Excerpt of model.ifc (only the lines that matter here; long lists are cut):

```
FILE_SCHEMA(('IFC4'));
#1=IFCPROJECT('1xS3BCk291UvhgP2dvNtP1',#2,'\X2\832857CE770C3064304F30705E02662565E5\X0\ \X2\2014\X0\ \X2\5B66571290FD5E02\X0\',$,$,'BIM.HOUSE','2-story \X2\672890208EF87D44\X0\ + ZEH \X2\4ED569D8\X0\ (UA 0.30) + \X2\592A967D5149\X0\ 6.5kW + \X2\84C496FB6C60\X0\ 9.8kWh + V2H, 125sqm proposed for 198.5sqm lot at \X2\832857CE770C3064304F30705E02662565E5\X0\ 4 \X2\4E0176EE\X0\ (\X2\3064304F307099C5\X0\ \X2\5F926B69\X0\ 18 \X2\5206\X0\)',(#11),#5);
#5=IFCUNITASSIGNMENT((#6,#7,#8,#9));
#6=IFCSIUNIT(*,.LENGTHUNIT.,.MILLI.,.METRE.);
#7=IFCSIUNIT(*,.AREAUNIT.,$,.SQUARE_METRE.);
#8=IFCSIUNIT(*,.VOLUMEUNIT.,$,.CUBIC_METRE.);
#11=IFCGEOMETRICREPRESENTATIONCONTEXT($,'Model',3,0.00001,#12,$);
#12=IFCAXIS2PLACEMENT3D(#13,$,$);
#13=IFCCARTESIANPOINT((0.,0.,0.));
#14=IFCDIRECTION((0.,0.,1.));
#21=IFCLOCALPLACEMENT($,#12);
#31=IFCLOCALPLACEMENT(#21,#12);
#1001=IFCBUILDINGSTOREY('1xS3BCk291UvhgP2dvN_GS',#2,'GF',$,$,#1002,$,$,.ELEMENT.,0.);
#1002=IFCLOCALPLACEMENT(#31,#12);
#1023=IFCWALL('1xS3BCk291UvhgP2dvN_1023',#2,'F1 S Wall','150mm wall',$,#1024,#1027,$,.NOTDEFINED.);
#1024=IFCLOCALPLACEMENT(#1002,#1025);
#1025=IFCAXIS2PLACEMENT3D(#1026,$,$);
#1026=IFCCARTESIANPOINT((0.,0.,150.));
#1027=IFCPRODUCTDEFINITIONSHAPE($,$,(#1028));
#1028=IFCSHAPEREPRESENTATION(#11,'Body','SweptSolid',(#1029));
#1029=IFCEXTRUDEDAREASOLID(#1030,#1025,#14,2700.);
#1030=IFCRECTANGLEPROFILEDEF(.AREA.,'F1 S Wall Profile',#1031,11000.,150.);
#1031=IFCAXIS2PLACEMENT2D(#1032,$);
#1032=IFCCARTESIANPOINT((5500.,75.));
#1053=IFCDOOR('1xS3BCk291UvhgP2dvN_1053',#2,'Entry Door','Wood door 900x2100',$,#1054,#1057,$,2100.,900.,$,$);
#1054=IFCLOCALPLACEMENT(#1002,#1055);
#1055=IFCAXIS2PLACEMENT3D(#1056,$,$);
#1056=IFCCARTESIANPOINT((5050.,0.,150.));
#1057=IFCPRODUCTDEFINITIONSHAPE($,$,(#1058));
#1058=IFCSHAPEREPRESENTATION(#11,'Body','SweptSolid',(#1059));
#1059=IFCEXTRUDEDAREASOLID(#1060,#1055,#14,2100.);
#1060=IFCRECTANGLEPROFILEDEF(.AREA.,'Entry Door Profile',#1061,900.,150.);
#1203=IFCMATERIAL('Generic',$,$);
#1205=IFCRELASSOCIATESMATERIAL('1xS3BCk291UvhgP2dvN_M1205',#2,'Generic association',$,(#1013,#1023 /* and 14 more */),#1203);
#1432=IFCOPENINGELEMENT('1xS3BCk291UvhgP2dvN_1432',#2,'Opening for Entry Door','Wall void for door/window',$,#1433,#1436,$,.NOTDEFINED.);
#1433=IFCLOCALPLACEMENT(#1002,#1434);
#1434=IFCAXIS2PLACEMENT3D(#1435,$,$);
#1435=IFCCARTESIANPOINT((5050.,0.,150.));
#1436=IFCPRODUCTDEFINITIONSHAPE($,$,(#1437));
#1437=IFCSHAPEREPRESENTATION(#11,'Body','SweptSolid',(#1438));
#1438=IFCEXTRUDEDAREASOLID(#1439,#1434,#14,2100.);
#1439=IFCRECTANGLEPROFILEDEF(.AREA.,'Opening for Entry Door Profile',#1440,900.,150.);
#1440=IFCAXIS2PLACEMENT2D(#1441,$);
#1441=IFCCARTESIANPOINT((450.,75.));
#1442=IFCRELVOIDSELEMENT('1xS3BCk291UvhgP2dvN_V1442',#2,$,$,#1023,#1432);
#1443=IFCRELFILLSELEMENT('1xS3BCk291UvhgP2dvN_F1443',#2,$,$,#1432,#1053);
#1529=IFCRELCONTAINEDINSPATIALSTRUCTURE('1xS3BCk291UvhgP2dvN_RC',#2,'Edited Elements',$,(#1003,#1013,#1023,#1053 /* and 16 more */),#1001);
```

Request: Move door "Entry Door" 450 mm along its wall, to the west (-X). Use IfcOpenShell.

```python
import ifcopenshell
import ifcopenshell.api.geometry
import ifcopenshell.util.placement

model = ifcopenshell.open("model.ifc")

door = model.by_guid("1xS3BCk291UvhgP2dvN_1053")
opening = door.FillsVoids[0].RelatingOpeningElement
wall = opening.VoidsElements[0].RelatingBuildingElement

wall_matrix = ifcopenshell.util.placement.get_local_placement(wall.ObjectPlacement)
shift = wall_matrix[:3, 0] * -450.0
before = ifcopenshell.util.placement.get_local_placement(door.ObjectPlacement)[:3, 3].copy()

# The door is not placed relative to its opening, so move both.
for product in (opening, door):
    matrix = ifcopenshell.util.placement.get_local_placement(product.ObjectPlacement)
    matrix[:3, 3] += shift
    ifcopenshell.api.geometry.edit_object_placement(model, product=product, matrix=matrix, is_si=False)

after = ifcopenshell.util.placement.get_local_placement(door.ObjectPlacement)[:3, 3]
print("door moved by", (after - before).round(3) + 0.0)

model.write("model_edited.ifc")
```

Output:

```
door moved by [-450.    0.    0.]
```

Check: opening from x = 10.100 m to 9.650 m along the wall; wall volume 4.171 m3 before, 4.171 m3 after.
